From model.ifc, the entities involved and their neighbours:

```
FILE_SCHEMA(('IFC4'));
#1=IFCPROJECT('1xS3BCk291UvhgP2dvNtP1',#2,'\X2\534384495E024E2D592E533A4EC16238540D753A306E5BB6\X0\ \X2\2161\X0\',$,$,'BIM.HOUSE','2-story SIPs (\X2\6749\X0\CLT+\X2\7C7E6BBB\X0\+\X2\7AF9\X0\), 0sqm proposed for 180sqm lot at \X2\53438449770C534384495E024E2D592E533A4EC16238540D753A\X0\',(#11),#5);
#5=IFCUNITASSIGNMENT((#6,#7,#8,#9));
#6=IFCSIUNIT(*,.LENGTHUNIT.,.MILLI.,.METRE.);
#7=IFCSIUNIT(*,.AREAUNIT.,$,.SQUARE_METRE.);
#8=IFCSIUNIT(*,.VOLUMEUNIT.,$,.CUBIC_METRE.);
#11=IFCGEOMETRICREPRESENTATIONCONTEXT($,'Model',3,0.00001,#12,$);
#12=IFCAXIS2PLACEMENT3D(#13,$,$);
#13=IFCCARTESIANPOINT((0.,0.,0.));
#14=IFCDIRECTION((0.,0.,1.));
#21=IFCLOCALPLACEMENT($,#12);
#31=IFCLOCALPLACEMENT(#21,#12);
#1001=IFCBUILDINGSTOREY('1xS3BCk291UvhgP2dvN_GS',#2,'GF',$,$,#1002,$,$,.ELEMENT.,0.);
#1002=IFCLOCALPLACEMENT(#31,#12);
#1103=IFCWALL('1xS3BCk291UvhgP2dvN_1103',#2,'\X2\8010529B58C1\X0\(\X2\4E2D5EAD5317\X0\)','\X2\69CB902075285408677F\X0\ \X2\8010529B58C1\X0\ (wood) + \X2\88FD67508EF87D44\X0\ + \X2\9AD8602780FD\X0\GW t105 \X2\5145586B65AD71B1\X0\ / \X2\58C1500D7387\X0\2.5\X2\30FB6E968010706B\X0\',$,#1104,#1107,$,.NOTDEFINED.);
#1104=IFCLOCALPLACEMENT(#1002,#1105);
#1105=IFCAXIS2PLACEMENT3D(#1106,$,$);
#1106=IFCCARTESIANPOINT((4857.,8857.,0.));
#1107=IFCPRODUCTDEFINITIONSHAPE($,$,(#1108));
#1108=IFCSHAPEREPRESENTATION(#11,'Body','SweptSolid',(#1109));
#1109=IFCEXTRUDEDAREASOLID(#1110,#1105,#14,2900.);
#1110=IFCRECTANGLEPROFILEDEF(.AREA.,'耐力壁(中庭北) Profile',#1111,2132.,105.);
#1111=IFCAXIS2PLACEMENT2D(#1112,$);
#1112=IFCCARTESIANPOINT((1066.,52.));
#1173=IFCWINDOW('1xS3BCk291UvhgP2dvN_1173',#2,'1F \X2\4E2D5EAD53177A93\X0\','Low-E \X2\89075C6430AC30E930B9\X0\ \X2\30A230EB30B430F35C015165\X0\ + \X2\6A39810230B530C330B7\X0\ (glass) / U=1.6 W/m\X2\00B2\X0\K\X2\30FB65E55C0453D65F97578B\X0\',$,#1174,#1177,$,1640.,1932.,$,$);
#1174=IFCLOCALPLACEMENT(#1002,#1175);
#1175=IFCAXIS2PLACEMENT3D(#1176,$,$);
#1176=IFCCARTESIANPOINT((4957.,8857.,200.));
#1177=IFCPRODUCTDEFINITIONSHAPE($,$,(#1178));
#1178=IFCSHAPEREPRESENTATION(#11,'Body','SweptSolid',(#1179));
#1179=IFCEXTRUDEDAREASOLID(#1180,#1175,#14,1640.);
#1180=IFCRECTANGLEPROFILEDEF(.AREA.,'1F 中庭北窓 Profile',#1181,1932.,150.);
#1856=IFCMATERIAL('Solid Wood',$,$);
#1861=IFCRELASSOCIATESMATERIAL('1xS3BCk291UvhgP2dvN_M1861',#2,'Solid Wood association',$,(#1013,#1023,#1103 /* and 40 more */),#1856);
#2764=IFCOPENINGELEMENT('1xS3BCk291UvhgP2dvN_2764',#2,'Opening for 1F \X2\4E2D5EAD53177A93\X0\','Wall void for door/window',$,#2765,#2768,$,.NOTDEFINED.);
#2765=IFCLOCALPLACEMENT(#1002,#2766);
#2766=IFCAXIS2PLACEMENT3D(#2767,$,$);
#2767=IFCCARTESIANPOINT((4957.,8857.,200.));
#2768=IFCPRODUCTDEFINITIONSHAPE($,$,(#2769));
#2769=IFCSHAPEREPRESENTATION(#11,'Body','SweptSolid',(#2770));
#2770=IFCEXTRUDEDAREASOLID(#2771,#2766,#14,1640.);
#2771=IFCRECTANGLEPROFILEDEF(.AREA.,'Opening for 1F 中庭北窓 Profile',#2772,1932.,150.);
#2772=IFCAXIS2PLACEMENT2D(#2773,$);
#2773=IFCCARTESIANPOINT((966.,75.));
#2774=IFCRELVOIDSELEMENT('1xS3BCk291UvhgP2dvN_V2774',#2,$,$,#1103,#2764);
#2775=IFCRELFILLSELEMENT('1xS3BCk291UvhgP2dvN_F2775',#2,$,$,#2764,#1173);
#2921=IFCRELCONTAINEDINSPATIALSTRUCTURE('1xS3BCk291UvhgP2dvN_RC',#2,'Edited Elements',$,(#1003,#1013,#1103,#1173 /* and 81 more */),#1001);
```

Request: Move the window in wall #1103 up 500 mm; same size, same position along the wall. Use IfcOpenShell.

```python
import numpy as np
import ifcopenshell
import ifcopenshell.api.geometry
import ifcopenshell.util.placement
import ifcopenshell.util.unit

model = ifcopenshell.open("model.ifc")
unit_scale = ifcopenshell.util.unit.calculate_unit_scale(model)

window = model.by_guid("1xS3BCk291UvhgP2dvN_1173")
opening = window.FillsVoids[0].RelatingOpeningElement
dz = 0.5 / unit_scale

shift = np.array([0.0, 0.0, dz])
# The window is not placed relative to its opening, so move both.
for product in (opening, window):
    matrix = ifcopenshell.util.placement.get_local_placement(product.ObjectPlacement)
    matrix[:3, 3] += shift
    ifcopenshell.api.geometry.edit_object_placement(model, product=product, matrix=matrix, is_si=False)

print(f"moved by {dz * unit_scale:+.3f} m")

model.write("model_v2.ifc")
```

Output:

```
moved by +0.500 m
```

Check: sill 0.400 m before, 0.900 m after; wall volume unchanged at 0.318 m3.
